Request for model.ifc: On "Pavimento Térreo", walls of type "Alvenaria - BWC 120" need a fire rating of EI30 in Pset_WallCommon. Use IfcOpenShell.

First a look at what the model holds.

```python
import ifcopenshell
import ifcopenshell.util.element

model = ifcopenshell.open("model.ifc")
print(model.schema)
storey = next(s for s in model.by_type("IfcBuildingStorey") if s.Name == "Pavimento Térreo")
walls = [e for e in ifcopenshell.util.element.get_decomposition(storey) if e.is_a("IfcWall")]
seen = {}
for e in walls:
    element_type = ifcopenshell.util.element.get_type(e)
    key = (element_type.Name if element_type != e and element_type else None, ifcopenshell.util.element.get_pset(e, "Pset_WallCommon", "FireRating"))
    seen[key] = seen.get(key, 0) + 1
for (name, value), count in sorted(seen.items(), key=str):
    print(count, "x", name, "|", value)
```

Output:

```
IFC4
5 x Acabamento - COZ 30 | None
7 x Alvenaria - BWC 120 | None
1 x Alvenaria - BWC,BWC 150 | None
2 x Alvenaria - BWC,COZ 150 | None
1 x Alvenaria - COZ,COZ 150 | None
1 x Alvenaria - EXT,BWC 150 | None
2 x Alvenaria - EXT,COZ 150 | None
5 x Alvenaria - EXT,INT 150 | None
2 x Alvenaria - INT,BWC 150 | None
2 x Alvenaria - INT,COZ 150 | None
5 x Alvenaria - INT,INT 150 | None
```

```python
import ifcopenshell
import ifcopenshell.api.pset
import ifcopenshell.util.element

model = ifcopenshell.open("model.ifc")

storey = next(s for s in model.by_type("IfcBuildingStorey") if s.Name == "Pavimento Térreo")
walls = [e for e in ifcopenshell.util.element.get_decomposition(storey) if e.is_a("IfcWall")]

count = 0
for e in walls:
    element_type = ifcopenshell.util.element.get_type(e)
    if element_type in (None, e) or element_type.Name != "Alvenaria - BWC 120":
        continue
    # add_pset returns the element's existing set when there is one.
    pset = ifcopenshell.api.pset.add_pset(model, product=e, name="Pset_WallCommon")
    ifcopenshell.api.pset.edit_pset(model, pset=pset, properties={"FireRating": "EI30"})
    count += 1

print(count, "walls updated")

model.write("model_v2.ifc")
```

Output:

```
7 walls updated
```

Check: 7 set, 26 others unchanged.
